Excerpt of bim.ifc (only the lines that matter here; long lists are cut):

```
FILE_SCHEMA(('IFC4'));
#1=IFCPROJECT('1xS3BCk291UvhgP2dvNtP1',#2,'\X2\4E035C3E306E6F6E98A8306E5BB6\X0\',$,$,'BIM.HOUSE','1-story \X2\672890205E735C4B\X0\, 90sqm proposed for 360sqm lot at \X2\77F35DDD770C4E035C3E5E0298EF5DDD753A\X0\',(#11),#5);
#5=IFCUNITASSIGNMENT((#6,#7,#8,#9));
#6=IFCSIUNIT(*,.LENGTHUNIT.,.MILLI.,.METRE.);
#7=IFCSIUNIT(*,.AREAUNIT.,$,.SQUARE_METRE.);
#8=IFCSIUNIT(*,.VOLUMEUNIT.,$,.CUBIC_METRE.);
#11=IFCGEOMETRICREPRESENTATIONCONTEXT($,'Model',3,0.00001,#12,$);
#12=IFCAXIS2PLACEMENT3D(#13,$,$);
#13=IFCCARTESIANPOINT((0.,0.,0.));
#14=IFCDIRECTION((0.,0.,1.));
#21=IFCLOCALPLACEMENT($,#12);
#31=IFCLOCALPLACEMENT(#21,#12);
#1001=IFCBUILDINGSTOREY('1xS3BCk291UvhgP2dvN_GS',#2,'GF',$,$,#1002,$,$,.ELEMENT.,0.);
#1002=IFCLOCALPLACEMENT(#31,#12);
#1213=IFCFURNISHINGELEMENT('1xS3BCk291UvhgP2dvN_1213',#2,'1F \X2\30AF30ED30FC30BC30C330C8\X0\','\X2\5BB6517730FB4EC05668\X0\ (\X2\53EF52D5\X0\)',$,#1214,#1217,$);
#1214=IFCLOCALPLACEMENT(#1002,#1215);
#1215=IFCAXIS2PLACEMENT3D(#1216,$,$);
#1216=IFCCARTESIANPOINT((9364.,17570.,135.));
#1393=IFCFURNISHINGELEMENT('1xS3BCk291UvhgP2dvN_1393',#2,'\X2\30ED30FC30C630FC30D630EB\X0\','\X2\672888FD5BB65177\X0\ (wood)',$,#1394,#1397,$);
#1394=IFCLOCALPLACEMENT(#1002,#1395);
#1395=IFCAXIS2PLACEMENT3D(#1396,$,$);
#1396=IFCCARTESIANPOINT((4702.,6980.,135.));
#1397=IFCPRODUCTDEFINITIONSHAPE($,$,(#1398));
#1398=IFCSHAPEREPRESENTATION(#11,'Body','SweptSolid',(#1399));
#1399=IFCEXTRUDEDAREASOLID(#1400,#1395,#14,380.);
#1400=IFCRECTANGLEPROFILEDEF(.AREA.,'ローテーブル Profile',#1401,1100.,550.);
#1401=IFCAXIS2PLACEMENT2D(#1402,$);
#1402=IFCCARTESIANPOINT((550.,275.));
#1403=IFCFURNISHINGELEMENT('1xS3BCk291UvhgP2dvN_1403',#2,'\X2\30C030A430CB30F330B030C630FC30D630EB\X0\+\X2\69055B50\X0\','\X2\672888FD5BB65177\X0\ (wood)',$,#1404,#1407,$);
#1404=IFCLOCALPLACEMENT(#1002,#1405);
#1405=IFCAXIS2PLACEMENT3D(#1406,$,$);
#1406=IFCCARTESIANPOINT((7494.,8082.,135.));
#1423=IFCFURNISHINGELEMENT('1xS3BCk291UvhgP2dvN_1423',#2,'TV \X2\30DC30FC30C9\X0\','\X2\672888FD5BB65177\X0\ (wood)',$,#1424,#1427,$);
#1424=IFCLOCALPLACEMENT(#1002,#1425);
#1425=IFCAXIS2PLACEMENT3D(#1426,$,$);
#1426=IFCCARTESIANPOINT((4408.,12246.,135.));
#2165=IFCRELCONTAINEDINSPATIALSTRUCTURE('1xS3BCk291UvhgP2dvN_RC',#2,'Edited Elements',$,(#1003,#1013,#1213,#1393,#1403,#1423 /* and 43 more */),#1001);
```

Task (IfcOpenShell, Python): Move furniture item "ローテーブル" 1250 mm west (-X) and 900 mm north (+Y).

```python
import ifcopenshell
import ifcopenshell.api.geometry
import ifcopenshell.util.placement

model = ifcopenshell.open("bim.ifc")

item = model.by_id(1393)
matrix = ifcopenshell.util.placement.get_local_placement(item.ObjectPlacement)
matrix[0, 3] -= 1250.0
matrix[1, 3] += 900.0
ifcopenshell.api.geometry.edit_object_placement(model, product=item, matrix=matrix, is_si=False)

print(ifcopenshell.util.placement.get_local_placement(item.ObjectPlacement).round(3) + 0.0)

model.write("bim_updated.ifc")
```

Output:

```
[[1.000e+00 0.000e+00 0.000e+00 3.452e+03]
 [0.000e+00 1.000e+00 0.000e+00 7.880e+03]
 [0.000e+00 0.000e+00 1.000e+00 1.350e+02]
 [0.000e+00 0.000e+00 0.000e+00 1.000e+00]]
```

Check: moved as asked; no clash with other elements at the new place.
